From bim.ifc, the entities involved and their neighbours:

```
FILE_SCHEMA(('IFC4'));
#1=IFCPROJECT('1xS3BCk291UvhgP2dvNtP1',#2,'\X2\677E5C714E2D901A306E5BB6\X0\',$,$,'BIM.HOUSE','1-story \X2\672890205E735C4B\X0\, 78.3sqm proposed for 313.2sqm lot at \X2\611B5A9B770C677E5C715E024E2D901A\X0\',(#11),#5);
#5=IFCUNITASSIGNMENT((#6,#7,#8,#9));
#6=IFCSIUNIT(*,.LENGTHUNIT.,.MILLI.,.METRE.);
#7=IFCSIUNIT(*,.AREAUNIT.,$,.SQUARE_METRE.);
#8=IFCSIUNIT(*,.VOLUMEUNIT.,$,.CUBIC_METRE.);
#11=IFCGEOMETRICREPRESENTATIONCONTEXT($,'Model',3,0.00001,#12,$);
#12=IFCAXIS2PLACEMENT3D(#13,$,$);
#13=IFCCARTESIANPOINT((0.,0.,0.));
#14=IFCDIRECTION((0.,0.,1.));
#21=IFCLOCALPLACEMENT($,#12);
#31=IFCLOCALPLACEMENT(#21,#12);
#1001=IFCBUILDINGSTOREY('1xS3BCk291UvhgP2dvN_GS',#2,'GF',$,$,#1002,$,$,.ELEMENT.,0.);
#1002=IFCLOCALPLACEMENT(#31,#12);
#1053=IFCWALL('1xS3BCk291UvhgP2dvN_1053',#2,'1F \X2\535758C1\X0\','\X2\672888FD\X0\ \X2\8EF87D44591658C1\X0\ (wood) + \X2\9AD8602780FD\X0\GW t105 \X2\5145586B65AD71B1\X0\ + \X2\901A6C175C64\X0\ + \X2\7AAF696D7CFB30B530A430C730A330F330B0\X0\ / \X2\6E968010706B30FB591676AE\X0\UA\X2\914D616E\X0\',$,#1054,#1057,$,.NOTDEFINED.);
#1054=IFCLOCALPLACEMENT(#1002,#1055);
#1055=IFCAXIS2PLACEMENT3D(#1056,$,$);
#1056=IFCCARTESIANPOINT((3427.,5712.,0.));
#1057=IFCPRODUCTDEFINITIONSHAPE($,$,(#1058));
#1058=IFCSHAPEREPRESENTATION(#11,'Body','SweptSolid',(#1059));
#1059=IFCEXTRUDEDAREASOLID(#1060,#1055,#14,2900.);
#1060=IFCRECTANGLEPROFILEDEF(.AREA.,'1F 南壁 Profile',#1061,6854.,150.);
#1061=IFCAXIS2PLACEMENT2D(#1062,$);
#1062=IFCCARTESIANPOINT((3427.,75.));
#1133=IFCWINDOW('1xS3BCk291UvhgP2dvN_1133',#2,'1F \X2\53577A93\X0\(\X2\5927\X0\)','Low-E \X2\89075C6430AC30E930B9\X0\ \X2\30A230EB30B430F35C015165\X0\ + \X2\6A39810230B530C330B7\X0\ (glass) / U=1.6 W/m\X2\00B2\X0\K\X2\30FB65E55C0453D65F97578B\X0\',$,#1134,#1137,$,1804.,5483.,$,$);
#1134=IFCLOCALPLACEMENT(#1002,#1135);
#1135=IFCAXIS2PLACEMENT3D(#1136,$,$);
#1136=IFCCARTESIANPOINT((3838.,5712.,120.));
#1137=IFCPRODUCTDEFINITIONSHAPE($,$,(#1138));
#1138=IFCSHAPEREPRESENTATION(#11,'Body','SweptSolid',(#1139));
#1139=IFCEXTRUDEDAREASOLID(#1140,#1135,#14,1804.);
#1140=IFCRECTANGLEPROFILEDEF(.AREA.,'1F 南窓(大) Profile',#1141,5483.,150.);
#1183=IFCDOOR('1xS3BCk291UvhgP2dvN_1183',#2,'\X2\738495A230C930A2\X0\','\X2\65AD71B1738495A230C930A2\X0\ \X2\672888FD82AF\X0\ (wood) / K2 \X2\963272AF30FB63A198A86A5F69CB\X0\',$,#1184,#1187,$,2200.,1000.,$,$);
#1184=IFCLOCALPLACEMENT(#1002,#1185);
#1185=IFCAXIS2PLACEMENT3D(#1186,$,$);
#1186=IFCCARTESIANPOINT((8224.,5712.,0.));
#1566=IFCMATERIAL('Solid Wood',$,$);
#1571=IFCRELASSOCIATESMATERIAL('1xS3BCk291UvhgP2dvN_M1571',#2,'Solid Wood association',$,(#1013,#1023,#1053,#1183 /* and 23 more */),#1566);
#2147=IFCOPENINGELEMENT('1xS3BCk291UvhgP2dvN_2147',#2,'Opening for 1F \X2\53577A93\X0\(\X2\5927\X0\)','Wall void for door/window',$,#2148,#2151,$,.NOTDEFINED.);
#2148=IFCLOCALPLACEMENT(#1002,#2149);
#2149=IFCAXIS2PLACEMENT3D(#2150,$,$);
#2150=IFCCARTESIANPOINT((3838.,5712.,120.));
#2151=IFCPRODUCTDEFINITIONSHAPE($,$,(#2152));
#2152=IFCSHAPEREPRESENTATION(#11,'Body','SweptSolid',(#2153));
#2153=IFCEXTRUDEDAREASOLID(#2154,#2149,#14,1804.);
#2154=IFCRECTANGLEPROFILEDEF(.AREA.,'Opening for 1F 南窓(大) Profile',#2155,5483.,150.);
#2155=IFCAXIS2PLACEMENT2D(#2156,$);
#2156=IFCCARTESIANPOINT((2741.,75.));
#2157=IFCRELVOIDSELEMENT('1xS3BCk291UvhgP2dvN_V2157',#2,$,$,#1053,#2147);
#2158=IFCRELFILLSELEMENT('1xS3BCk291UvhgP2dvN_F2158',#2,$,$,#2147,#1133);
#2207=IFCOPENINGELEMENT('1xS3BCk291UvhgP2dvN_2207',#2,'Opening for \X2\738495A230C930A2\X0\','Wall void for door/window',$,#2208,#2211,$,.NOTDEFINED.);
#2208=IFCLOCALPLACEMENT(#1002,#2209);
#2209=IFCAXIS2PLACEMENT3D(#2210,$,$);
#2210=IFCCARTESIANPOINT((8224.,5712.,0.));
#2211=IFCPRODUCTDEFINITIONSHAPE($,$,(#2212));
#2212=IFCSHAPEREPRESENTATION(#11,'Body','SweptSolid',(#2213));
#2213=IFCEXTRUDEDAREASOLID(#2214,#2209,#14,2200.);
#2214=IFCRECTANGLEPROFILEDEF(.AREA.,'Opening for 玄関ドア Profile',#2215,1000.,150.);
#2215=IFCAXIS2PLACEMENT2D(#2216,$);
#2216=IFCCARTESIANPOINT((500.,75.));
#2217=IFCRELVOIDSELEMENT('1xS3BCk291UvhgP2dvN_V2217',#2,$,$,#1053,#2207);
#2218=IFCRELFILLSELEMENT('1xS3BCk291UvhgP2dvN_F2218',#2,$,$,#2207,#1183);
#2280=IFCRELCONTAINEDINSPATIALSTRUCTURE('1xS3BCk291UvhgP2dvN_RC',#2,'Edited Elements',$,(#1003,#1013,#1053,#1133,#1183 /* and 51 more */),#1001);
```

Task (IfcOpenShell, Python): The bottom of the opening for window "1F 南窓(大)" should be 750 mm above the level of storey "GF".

```python
import numpy as np
import ifcopenshell
import ifcopenshell.api.geometry
import ifcopenshell.geom
import ifcopenshell.util.element
import ifcopenshell.util.placement
import ifcopenshell.util.shape
import ifcopenshell.util.unit

model = ifcopenshell.open("bim.ifc")
unit_scale = ifcopenshell.util.unit.calculate_unit_scale(model)

window = model.by_guid("1xS3BCk291UvhgP2dvN_1133")
opening = window.FillsVoids[0].RelatingOpeningElement
storey = ifcopenshell.util.element.get_container(window, ifc_class="IfcBuildingStorey")
level = ifcopenshell.util.placement.get_local_placement(storey.ObjectPlacement)[2, 3]

# The opening's origin need not be at the sill, so measure its lowest point.
shape = ifcopenshell.geom.create_shape(ifcopenshell.geom.settings(), opening)
bottom = ifcopenshell.util.shape.get_shape_bottom_elevation(shape, shape.geometry) / unit_scale
dz = level + 0.75 / unit_scale - bottom

shift = np.array([0.0, 0.0, dz])
# The window is not placed relative to its opening, so move both.
for product in (opening, window):
    matrix = ifcopenshell.util.placement.get_local_placement(product.ObjectPlacement)
    matrix[:3, 3] += shift
    ifcopenshell.api.geometry.edit_object_placement(model, product=product, matrix=matrix, is_si=False)

print(f"moved by {dz * unit_scale:+.3f} m")

model.write("bim_rev.ifc")
```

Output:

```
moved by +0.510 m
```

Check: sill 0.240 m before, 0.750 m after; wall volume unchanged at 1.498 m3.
